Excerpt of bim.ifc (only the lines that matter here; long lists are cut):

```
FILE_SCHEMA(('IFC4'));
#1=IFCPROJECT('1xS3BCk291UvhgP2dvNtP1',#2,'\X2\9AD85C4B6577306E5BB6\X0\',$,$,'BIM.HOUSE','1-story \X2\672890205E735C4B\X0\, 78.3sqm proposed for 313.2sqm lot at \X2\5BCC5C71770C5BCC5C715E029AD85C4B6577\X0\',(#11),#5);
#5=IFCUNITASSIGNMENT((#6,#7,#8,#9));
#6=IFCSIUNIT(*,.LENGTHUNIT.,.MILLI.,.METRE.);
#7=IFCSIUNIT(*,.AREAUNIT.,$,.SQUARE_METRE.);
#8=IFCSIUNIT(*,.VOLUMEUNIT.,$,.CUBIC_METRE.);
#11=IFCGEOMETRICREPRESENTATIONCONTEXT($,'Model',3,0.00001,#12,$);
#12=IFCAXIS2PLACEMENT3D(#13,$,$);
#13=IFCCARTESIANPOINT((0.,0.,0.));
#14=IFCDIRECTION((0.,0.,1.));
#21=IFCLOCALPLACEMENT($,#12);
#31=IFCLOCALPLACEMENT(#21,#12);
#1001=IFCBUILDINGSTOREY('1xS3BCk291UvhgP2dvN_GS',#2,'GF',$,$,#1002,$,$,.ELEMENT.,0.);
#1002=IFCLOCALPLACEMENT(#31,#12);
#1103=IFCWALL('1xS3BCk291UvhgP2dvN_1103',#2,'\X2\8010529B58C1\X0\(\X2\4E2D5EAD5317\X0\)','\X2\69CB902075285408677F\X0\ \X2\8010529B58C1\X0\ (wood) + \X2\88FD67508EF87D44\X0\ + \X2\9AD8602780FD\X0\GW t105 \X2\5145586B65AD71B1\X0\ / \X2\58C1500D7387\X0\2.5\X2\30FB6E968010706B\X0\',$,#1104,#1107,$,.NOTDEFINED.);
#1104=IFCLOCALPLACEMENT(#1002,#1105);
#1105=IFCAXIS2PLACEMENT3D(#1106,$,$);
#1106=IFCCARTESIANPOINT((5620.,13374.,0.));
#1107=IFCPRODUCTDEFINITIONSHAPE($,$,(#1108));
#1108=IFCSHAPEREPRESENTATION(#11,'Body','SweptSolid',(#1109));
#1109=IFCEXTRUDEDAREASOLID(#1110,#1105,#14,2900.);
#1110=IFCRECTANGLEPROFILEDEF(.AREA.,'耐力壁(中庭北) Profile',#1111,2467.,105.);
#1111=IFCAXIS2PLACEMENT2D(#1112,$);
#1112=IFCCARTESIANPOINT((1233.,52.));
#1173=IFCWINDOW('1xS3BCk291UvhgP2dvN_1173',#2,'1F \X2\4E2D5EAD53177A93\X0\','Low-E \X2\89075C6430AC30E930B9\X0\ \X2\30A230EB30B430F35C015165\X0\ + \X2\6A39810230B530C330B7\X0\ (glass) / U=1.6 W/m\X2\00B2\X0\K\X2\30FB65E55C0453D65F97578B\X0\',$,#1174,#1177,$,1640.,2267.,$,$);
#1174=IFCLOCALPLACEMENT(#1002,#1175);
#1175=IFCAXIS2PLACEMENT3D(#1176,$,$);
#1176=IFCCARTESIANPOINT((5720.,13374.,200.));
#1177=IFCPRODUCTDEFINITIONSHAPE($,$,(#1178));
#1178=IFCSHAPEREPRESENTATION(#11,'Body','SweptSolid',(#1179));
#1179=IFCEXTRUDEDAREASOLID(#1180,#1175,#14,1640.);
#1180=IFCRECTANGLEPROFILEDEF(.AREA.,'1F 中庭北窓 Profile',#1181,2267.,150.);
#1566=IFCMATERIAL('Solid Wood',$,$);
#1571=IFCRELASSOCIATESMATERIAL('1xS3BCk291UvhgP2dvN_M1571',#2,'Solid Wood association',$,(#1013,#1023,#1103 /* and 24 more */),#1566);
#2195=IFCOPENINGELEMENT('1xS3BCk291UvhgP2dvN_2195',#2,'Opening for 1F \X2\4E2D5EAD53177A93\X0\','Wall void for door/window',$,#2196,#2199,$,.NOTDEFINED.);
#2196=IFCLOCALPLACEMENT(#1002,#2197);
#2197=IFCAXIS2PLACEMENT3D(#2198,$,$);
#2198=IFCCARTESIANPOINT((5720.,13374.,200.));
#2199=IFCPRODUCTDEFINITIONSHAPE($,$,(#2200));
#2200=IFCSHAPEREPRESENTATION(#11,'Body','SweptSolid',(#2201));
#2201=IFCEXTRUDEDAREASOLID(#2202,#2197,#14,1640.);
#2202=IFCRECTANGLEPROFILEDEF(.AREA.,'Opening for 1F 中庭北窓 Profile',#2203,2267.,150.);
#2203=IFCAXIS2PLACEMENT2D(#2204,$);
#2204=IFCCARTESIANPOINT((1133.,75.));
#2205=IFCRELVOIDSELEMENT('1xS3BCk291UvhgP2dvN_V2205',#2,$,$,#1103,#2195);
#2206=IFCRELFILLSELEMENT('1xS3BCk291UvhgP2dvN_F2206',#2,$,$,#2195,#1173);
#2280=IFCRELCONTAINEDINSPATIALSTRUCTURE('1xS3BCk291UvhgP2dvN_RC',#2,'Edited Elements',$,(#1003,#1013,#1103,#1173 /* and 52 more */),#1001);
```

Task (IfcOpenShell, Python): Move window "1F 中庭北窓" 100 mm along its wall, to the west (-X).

```python
import ifcopenshell
import ifcopenshell.api.geometry
import ifcopenshell.util.placement

model = ifcopenshell.open("bim.ifc")

window = model.by_id(1173)
opening = window.FillsVoids[0].RelatingOpeningElement
wall = opening.VoidsElements[0].RelatingBuildingElement

wall_matrix = ifcopenshell.util.placement.get_local_placement(wall.ObjectPlacement)
shift = wall_matrix[:3, 0] * -100.0
before = ifcopenshell.util.placement.get_local_placement(window.ObjectPlacement)[:3, 3].copy()

# The window is not placed relative to its opening, so move both.
for product in (opening, window):
    matrix = ifcopenshell.util.placement.get_local_placement(product.ObjectPlacement)
    matrix[:3, 3] += shift
    ifcopenshell.api.geometry.edit_object_placement(model, product=product, matrix=matrix, is_si=False)

after = ifcopenshell.util.placement.get_local_placement(window.ObjectPlacement)[:3, 3]
print("window moved by", (after - before).round(3) + 0.0)

model.write("bim_updated.ifc")
```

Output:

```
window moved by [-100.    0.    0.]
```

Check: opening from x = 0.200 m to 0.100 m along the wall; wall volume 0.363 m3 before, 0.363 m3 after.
